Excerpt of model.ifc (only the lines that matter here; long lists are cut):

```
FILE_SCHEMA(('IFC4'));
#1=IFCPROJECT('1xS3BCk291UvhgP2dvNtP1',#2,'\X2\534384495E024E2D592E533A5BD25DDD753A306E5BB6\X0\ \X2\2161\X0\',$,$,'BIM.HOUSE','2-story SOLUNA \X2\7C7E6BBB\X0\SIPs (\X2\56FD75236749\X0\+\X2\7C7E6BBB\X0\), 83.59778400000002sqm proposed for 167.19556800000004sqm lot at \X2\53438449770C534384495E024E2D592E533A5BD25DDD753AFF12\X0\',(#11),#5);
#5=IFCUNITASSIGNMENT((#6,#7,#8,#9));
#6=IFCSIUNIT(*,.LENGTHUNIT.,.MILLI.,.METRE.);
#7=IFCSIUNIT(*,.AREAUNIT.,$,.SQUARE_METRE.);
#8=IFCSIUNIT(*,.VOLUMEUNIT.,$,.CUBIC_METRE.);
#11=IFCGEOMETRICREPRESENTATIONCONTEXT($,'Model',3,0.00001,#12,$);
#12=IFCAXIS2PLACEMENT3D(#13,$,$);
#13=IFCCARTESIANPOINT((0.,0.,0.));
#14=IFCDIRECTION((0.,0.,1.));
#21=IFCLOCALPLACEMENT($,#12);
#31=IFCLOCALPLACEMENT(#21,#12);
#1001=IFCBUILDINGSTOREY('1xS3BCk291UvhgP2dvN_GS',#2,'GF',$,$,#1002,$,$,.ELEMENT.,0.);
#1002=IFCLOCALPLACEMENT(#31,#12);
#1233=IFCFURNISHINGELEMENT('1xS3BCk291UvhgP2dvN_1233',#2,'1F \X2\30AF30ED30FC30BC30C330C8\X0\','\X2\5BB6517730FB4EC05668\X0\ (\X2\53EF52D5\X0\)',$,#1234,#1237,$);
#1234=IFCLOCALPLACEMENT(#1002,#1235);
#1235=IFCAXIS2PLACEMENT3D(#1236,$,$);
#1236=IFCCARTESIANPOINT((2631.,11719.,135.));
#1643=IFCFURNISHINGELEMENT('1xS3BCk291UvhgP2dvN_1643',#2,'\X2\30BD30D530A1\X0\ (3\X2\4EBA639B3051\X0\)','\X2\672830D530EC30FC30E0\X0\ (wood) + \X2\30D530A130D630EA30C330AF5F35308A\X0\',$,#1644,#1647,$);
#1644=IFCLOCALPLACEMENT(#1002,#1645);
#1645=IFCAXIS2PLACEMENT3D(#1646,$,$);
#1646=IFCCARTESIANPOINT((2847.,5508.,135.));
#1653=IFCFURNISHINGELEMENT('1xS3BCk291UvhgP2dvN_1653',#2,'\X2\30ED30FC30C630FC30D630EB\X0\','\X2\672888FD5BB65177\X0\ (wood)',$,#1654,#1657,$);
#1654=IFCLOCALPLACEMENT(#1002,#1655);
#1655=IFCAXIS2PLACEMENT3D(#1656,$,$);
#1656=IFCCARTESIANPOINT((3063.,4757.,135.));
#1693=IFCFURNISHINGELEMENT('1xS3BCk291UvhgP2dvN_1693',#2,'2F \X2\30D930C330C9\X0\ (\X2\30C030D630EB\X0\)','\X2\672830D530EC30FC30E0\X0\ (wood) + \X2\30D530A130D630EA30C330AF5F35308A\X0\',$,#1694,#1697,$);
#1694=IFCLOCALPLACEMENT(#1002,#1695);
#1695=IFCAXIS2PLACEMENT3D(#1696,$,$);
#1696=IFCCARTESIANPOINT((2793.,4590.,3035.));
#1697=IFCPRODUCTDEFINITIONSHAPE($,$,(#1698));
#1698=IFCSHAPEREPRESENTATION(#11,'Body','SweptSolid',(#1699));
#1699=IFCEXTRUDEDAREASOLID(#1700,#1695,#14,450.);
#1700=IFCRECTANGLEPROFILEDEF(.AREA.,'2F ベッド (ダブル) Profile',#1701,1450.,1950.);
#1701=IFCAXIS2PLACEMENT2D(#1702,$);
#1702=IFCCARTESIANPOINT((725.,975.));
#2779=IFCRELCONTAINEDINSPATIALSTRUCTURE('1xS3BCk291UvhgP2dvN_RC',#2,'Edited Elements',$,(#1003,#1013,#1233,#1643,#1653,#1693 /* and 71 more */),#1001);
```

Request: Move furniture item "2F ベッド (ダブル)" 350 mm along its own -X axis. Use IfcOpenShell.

```python
import ifcopenshell
import ifcopenshell.api.geometry
import ifcopenshell.util.placement
import ifcopenshell.util.unit

model = ifcopenshell.open("model.ifc")
unit_scale = ifcopenshell.util.unit.calculate_unit_scale(model)

item = model.by_id(1693)
matrix = ifcopenshell.util.placement.get_local_placement(item.ObjectPlacement)
matrix[:3, 3] -= matrix[:3, 0] * 0.35 / unit_scale
ifcopenshell.api.geometry.edit_object_placement(model, product=item, matrix=matrix, is_si=False)

print(ifcopenshell.util.placement.get_local_placement(item.ObjectPlacement).round(3) + 0.0)

model.write("model_rev.ifc")
```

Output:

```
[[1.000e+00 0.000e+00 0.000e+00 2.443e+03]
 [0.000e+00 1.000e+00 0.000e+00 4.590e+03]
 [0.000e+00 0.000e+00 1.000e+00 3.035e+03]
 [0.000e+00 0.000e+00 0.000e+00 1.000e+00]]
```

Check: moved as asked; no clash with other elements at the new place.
